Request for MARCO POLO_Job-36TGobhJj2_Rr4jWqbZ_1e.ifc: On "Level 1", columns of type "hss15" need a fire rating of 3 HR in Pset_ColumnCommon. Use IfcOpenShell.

First a look at what the model holds.

```python
import ifcopenshell
import ifcopenshell.util.element

model = ifcopenshell.open("MARCO POLO_Job-36TGobhJj2_Rr4jWqbZ_1e.ifc")
print(model.schema)
storey = next(s for s in model.by_type("IfcBuildingStorey") if s.Name == "Level 1")
columns = [e for e in ifcopenshell.util.element.get_decomposition(storey) if e.is_a("IfcColumn")]
seen = {}
for e in columns:
    element_type = ifcopenshell.util.element.get_type(e)
    key = (element_type.Name if element_type != e and element_type else None, ifcopenshell.util.element.get_pset(e, "Pset_ColumnCommon", "FireRating"))
    seen[key] = seen.get(key, 0) + 1
for (name, value), count in sorted(seen.items(), key=str):
    print(count, "x", name, "|", value)
```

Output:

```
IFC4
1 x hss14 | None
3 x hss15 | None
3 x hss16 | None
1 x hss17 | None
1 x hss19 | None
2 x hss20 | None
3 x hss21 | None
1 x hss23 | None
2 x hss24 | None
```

```python
import ifcopenshell
import ifcopenshell.api.pset
import ifcopenshell.util.element

model = ifcopenshell.open("MARCO POLO_Job-36TGobhJj2_Rr4jWqbZ_1e.ifc")

storey = next(s for s in model.by_type("IfcBuildingStorey") if s.Name == "Level 1")
columns = [e for e in ifcopenshell.util.element.get_decomposition(storey) if e.is_a("IfcColumn")]

count = 0
for e in columns:
    element_type = ifcopenshell.util.element.get_type(e)
    if element_type in (None, e) or element_type.Name != "hss15":
        continue
    # add_pset returns the element's existing set when there is one.
    pset = ifcopenshell.api.pset.add_pset(model, product=e, name="Pset_ColumnCommon")
    ifcopenshell.api.pset.edit_pset(model, pset=pset, properties={"FireRating": "3 HR"})
    count += 1

print(count, "columns updated")

model.write("MARCO POLO_Job-36TGobhJj2_Rr4jWqbZ_1e_rev.ifc")
```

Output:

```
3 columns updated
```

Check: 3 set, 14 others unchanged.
